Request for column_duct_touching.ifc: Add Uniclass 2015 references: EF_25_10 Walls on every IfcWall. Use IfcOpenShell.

First a look at what the model holds.

```python
import ifcopenshell

model = ifcopenshell.open("column_duct_touching.ifc")
print(model.schema)
print("classifications:", [c.Name for c in model.by_type("IfcClassification")])
for ifc_class in ("IfcDoor", "IfcRoof", "IfcStair", "IfcWall", "IfcWindow"):
    print(ifc_class, len(model.by_type(ifc_class)))
```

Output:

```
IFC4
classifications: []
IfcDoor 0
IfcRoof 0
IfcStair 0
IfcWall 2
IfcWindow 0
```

```python
import ifcopenshell
import ifcopenshell.api.classification

model = ifcopenshell.open("column_duct_touching.ifc")

system = ifcopenshell.api.classification.add_classification(model, classification="Uniclass 2015")

codes = {
    "IfcWall": ("EF_25_10", "Walls"),
}
for ifc_class, (code, name) in codes.items():
    products = model.by_type(ifc_class)
    ifcopenshell.api.classification.add_reference(
        model, products=products, classification=system, identification=code, name=name
    )
    print(code, len(products))

model.write("column_duct_touching_v2.ifc")
```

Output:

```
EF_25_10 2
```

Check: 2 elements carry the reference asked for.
